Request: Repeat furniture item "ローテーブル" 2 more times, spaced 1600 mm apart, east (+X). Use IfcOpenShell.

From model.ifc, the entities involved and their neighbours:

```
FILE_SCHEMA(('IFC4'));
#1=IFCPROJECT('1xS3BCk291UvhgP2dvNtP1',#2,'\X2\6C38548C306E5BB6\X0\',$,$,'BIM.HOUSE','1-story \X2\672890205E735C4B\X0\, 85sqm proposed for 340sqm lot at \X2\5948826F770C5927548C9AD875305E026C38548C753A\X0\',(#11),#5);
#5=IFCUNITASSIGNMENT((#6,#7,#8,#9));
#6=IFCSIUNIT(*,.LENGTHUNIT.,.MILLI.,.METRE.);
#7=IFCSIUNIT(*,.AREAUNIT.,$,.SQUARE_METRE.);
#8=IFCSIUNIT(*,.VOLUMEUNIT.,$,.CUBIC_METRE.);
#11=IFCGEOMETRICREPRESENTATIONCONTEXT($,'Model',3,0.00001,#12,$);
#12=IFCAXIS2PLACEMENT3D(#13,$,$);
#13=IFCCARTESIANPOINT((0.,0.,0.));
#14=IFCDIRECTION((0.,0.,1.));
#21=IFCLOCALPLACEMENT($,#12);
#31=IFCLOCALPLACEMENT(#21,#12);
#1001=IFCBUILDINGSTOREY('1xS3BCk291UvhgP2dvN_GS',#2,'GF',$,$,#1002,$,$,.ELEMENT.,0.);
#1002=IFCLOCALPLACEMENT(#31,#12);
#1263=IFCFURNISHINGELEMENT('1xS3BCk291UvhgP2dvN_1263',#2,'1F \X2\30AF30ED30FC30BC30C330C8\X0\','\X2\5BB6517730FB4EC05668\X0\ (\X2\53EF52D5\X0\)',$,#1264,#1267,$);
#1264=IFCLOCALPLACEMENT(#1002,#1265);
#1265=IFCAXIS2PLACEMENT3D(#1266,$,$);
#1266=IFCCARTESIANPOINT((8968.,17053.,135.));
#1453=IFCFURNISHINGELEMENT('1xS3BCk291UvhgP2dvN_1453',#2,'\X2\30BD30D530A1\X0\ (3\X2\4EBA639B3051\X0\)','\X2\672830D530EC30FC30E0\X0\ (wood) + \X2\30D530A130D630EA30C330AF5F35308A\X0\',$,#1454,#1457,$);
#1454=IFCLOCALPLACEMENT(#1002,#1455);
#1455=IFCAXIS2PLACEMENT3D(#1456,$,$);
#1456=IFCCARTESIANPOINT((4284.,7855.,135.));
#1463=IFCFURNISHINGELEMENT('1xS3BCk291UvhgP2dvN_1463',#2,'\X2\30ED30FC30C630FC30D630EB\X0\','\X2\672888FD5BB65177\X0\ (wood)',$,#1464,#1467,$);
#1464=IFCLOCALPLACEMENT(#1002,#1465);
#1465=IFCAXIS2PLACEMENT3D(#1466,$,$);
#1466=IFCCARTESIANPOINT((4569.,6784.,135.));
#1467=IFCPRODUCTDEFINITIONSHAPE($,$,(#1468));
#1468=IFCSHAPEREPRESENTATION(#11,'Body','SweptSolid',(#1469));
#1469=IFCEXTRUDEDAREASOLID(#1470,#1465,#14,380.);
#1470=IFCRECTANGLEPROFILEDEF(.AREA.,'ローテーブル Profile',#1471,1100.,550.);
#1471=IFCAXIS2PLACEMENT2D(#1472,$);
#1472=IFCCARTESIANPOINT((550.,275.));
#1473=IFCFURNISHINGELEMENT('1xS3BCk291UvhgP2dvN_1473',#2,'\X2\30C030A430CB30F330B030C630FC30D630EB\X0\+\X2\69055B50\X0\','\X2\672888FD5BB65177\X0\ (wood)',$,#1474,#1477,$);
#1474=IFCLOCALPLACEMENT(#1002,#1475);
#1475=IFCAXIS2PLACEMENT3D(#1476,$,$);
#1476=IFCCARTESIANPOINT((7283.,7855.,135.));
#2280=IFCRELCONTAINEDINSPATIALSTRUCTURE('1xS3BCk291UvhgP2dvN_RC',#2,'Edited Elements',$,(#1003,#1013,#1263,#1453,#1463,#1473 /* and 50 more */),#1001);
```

```python
import numpy as np
import ifcopenshell
import ifcopenshell.api.geometry
import ifcopenshell.api.root
import ifcopenshell.util.element
import ifcopenshell.util.placement
import ifcopenshell.util.unit

model = ifcopenshell.open("model.ifc")
unit_scale = ifcopenshell.util.unit.calculate_unit_scale(model)


def reuse_history(source, copy):
    """copy_class also copies each property set's owner history, people and application; keep the originals."""
    for rel in copy.IsDefinedBy:
        if rel.is_a("IfcRelDefinesByProperties") and (history := rel.RelatingPropertyDefinition.OwnerHistory):
            rel.RelatingPropertyDefinition.OwnerHistory = source.OwnerHistory
            ifcopenshell.util.element.remove_deep2(model, history)


source = model.by_guid("1xS3BCk291UvhgP2dvN_1463")
base = ifcopenshell.util.placement.get_local_placement(source.ObjectPlacement)
step = np.array([1.0, 0.0, 0.0]) * 1.6 / unit_scale

for i in range(1, 3):
    copy = ifcopenshell.api.root.copy_class(model, product=source)
    copy.Representation = ifcopenshell.util.element.copy_deep(
        model, source.Representation, exclude=["IfcGeometricRepresentationContext", "IfcRepresentationMap"]
    )
    reuse_history(source, copy)
    matrix = base.copy()
    matrix[:3, 3] += i * step
    print("added at", matrix[:3, 3].round(3) + 0.0)
    ifcopenshell.api.geometry.edit_object_placement(model, product=copy, matrix=matrix, is_si=False)

model.write("model_rev.ifc")
```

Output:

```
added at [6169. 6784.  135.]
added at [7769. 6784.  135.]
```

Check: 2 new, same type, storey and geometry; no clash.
